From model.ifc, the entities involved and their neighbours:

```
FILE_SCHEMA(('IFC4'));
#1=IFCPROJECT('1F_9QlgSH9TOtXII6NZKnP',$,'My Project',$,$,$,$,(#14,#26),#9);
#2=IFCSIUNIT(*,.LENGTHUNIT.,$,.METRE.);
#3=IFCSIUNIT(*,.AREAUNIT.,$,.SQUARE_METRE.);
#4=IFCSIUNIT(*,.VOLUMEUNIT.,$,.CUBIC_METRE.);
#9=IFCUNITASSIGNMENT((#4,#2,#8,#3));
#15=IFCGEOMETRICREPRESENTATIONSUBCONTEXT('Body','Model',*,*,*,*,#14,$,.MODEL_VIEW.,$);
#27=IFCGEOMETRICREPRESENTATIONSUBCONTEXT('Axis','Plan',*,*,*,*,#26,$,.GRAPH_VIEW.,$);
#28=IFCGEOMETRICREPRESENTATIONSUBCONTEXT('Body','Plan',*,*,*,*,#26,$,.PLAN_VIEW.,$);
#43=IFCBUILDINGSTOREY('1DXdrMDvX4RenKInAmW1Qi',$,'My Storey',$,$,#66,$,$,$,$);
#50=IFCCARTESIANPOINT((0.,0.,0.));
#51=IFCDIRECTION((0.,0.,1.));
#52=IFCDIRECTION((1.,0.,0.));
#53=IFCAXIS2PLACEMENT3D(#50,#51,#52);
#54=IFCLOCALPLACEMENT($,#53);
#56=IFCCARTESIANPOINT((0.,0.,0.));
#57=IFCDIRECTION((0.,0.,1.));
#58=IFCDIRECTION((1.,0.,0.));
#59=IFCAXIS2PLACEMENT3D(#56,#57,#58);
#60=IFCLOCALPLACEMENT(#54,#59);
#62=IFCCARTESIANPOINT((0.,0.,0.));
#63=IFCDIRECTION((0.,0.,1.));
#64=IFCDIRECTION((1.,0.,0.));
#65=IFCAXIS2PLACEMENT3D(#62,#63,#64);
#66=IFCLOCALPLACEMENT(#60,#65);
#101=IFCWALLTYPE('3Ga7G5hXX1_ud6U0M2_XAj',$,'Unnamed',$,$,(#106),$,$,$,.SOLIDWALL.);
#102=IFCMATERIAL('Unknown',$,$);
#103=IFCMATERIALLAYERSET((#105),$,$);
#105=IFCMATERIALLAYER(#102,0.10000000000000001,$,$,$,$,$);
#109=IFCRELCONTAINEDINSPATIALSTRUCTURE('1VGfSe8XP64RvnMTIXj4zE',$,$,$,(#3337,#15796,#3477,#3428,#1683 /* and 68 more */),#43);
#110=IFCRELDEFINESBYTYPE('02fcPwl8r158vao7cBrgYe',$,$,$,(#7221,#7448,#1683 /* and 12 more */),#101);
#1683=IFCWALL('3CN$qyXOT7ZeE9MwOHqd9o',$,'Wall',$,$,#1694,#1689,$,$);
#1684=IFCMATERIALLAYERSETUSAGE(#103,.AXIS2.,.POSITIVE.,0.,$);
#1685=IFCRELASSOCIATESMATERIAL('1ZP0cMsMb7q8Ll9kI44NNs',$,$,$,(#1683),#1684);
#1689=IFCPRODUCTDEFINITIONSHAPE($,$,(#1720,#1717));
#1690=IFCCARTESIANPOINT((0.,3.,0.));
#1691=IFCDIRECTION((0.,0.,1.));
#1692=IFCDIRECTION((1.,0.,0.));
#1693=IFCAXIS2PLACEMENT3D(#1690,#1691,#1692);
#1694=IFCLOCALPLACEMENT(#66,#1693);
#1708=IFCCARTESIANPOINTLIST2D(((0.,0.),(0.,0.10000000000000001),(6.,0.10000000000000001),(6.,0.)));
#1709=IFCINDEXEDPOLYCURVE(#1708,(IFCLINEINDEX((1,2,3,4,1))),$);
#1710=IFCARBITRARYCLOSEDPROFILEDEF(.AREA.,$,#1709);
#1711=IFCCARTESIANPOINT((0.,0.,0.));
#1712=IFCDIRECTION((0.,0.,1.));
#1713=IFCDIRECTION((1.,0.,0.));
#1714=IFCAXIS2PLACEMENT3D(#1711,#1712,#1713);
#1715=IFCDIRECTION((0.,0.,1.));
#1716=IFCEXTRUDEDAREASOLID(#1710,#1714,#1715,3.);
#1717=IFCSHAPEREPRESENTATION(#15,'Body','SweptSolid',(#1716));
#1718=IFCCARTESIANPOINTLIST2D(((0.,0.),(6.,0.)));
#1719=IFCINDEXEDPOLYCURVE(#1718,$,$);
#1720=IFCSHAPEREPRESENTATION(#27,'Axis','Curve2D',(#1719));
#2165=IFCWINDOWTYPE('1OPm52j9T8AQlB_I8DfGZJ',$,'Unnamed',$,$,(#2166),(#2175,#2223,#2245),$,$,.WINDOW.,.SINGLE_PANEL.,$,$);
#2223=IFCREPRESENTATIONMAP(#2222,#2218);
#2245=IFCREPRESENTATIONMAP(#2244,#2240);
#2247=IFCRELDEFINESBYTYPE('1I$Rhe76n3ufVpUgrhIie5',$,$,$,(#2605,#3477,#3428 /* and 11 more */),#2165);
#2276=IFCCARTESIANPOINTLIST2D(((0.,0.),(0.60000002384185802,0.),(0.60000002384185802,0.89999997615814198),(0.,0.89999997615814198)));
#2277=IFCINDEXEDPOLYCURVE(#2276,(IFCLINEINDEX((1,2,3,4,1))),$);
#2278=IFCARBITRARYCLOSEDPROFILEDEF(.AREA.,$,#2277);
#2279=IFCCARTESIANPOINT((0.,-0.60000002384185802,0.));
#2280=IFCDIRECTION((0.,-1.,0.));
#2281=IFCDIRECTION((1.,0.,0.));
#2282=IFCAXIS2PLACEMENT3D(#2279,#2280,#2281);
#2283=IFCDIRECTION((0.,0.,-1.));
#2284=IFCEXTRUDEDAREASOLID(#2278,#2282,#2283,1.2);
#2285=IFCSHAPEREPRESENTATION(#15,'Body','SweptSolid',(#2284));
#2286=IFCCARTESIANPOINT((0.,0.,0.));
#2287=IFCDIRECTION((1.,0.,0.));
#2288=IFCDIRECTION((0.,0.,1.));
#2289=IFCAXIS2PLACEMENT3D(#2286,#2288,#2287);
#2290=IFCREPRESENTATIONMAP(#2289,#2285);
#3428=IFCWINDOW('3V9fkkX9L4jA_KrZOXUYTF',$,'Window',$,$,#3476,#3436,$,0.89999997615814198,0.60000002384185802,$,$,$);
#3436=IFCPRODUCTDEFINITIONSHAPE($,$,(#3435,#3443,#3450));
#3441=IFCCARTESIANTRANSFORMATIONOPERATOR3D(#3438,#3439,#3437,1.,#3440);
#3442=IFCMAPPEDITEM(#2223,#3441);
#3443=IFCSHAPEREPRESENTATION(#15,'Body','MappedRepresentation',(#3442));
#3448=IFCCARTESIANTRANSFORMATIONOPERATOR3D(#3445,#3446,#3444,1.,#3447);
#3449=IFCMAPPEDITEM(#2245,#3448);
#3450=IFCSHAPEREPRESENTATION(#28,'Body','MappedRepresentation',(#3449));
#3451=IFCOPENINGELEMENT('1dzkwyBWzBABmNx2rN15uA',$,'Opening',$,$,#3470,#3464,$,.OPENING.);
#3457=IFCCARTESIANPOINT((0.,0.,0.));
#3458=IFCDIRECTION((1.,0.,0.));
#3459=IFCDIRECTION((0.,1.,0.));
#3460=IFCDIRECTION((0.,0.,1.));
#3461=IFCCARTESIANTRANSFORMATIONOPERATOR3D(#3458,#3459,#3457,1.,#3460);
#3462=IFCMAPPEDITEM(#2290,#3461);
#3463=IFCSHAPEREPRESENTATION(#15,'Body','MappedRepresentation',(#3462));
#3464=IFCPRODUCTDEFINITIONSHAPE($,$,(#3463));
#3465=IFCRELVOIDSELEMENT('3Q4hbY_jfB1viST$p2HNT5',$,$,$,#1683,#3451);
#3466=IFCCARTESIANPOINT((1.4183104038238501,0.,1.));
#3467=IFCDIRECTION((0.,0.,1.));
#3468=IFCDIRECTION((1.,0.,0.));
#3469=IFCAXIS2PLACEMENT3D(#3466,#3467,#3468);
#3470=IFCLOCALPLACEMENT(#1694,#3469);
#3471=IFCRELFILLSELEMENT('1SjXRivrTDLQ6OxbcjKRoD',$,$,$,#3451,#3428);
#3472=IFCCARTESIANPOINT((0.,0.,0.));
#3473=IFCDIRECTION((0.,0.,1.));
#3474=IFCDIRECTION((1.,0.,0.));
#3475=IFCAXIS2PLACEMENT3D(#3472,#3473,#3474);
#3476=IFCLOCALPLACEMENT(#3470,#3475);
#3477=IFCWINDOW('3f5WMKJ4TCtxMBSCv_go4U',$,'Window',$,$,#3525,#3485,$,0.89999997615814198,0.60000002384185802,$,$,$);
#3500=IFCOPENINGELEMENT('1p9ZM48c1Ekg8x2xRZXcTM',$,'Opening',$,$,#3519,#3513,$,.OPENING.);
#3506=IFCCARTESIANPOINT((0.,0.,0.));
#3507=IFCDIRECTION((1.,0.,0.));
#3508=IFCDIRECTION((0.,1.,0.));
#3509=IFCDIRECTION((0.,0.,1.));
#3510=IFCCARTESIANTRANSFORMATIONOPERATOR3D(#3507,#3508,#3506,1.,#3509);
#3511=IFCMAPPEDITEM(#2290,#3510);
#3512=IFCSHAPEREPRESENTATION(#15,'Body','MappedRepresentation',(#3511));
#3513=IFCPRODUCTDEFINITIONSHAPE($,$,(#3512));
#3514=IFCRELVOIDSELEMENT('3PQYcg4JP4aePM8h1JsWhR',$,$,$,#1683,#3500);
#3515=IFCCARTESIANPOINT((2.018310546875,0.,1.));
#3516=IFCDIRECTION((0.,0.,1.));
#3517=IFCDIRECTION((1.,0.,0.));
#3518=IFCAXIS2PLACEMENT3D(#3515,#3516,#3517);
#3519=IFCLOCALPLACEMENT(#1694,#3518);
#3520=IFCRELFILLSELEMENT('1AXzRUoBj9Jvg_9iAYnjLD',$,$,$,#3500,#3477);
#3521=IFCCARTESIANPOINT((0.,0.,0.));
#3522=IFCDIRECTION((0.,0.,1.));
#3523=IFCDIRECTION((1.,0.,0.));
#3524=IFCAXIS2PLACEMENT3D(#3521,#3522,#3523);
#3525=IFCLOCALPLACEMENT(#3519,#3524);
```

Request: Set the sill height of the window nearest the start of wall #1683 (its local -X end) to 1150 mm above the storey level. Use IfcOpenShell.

```python
import numpy as np
import ifcopenshell
import ifcopenshell.api.geometry
import ifcopenshell.geom
import ifcopenshell.util.element
import ifcopenshell.util.placement
import ifcopenshell.util.shape
import ifcopenshell.util.unit

model = ifcopenshell.open("model.ifc")
unit_scale = ifcopenshell.util.unit.calculate_unit_scale(model)

window = model.by_guid("3V9fkkX9L4jA_KrZOXUYTF")
opening = window.FillsVoids[0].RelatingOpeningElement
storey = ifcopenshell.util.element.get_container(window, ifc_class="IfcBuildingStorey")
level = ifcopenshell.util.placement.get_local_placement(storey.ObjectPlacement)[2, 3]

# The opening's origin need not be at the sill, so measure its lowest point.
shape = ifcopenshell.geom.create_shape(ifcopenshell.geom.settings(), opening)
bottom = ifcopenshell.util.shape.get_shape_bottom_elevation(shape, shape.geometry) / unit_scale
dz = level + 1.15 / unit_scale - bottom

shift = np.array([0.0, 0.0, dz])
# The window is placed relative to its opening, so it follows when the opening moves.
matrix = ifcopenshell.util.placement.get_local_placement(opening.ObjectPlacement)
matrix[:3, 3] += shift
ifcopenshell.api.geometry.edit_object_placement(
    model, product=opening, matrix=matrix, is_si=False, should_transform_children=True
)

print(f"moved by {dz * unit_scale:+.3f} m")

model.write("model_edited.ifc")
```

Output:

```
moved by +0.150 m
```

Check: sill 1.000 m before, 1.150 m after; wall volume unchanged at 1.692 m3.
